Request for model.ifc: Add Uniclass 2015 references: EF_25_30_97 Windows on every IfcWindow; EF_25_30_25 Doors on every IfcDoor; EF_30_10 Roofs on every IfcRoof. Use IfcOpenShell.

First a look at what the model holds.

```python
import ifcopenshell

model = ifcopenshell.open("model.ifc")
print(model.schema)
print("classifications:", [c.Name for c in model.by_type("IfcClassification")])
for ifc_class in ("IfcDoor", "IfcRoof", "IfcStair", "IfcWall", "IfcWindow"):
    print(ifc_class, len(model.by_type(ifc_class)))
```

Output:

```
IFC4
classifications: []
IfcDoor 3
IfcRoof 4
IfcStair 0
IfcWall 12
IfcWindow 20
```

```python
import ifcopenshell
import ifcopenshell.api.classification

model = ifcopenshell.open("model.ifc")

system = ifcopenshell.api.classification.add_classification(model, classification="Uniclass 2015")

codes = {
    "IfcWindow": ("EF_25_30_97", "Windows"),
    "IfcDoor": ("EF_25_30_25", "Doors"),
    "IfcRoof": ("EF_30_10", "Roofs"),
}
for ifc_class, (code, name) in codes.items():
    products = model.by_type(ifc_class)
    ifcopenshell.api.classification.add_reference(
        model, products=products, classification=system, identification=code, name=name
    )
    print(code, len(products))

model.write("model_rev.ifc")
```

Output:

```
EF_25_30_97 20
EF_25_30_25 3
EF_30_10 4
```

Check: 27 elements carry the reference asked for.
